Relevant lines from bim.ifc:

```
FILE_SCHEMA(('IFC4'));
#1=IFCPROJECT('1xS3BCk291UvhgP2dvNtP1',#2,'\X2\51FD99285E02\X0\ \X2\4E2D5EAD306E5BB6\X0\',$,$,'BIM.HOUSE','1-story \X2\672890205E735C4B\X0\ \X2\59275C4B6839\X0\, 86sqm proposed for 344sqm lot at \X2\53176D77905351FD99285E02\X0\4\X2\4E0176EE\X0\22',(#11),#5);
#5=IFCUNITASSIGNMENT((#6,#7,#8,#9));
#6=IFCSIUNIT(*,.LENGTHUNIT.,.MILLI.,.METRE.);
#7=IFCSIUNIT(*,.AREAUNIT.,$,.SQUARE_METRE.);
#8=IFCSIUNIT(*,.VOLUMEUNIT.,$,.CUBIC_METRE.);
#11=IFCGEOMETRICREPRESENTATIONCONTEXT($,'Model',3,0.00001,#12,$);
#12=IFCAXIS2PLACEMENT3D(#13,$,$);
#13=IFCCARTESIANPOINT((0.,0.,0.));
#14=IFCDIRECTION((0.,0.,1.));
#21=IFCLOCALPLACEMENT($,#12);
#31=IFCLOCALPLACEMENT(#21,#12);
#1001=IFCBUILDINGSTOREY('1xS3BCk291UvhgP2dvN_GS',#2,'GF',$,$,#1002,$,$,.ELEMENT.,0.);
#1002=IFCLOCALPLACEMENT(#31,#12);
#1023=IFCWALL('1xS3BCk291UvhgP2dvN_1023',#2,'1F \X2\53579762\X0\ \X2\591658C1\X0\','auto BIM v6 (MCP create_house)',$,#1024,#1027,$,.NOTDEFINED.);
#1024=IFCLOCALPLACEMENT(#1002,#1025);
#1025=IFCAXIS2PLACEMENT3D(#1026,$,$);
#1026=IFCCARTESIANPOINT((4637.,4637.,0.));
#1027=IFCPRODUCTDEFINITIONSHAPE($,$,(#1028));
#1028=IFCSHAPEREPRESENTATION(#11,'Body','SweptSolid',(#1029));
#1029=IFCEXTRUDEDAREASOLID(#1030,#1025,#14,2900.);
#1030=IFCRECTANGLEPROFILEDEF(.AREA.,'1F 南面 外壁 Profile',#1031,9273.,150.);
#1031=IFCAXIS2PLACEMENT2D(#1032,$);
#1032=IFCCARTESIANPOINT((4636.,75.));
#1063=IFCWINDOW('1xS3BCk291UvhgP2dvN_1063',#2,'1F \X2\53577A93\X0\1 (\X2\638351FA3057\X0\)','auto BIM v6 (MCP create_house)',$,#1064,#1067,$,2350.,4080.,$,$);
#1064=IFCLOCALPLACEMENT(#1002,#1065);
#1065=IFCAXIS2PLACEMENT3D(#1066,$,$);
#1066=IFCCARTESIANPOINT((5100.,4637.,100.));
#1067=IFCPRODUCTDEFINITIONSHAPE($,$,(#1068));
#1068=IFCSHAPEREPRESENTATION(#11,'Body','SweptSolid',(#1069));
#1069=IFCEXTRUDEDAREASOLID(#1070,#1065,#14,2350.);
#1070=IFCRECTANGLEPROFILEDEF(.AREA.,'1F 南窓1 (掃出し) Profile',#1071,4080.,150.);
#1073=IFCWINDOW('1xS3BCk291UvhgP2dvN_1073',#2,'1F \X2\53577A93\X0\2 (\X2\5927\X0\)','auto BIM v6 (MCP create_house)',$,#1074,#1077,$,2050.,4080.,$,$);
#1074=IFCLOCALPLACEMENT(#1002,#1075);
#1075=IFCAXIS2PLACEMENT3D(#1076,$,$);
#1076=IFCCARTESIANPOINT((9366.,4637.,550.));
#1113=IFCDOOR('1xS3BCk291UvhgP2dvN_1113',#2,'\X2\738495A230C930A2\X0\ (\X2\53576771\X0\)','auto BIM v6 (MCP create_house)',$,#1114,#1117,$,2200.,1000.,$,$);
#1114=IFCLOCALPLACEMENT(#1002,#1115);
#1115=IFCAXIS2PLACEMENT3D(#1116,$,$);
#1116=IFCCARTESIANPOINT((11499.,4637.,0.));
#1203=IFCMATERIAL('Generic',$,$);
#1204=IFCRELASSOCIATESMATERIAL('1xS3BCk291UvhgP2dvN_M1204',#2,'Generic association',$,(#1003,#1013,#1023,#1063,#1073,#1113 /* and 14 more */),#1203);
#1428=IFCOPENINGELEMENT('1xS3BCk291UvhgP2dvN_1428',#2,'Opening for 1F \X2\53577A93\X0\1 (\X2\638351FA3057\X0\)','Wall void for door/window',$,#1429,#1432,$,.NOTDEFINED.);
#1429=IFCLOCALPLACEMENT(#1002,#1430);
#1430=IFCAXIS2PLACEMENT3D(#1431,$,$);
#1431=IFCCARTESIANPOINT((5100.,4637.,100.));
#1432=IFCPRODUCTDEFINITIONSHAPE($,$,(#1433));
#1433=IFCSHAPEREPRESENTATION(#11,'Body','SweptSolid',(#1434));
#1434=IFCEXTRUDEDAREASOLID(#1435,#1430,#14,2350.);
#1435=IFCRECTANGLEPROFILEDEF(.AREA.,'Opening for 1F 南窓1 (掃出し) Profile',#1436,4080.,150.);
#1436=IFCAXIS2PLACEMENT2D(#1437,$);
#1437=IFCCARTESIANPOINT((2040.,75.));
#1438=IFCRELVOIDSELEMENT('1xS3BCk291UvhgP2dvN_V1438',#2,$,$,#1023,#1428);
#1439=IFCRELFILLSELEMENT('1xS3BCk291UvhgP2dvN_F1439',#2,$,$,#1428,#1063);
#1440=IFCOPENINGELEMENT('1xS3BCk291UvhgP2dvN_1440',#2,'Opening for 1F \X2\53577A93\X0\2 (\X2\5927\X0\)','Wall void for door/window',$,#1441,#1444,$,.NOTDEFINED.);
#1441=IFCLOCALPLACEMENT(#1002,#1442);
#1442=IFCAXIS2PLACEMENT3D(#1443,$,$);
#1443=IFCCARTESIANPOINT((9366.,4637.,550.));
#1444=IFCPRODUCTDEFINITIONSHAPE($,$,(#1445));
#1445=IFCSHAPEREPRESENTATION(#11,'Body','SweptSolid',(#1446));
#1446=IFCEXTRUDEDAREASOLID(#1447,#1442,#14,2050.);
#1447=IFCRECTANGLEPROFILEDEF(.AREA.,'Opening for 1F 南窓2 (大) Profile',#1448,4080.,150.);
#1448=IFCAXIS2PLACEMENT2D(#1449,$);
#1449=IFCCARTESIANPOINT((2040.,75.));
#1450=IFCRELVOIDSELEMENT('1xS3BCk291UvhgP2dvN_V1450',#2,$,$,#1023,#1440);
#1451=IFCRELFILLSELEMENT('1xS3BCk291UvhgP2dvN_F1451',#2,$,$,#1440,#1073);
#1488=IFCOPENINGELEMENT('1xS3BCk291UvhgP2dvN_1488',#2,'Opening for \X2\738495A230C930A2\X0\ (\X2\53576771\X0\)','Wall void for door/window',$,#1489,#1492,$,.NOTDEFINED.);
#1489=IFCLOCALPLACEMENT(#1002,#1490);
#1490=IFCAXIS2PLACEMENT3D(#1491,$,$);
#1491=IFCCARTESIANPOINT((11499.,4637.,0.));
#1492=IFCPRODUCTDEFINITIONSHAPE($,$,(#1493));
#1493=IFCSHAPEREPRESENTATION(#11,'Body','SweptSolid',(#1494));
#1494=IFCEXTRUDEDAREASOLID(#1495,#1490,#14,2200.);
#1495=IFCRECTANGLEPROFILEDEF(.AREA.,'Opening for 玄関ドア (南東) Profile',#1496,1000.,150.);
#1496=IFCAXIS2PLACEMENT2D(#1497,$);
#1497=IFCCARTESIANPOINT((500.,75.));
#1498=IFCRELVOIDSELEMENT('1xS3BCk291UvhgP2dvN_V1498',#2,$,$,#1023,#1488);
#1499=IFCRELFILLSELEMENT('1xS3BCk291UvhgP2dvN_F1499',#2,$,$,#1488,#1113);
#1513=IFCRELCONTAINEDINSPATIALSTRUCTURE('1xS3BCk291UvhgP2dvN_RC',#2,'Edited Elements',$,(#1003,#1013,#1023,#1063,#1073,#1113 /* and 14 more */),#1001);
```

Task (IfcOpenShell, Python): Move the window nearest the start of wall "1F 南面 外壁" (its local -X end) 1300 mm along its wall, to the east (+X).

```python
import ifcopenshell
import ifcopenshell.api.geometry
import ifcopenshell.util.placement
import ifcopenshell.util.unit

model = ifcopenshell.open("bim.ifc")
unit_scale = ifcopenshell.util.unit.calculate_unit_scale(model)

window = model.by_id(1063)
opening = window.FillsVoids[0].RelatingOpeningElement
wall = opening.VoidsElements[0].RelatingBuildingElement

wall_matrix = ifcopenshell.util.placement.get_local_placement(wall.ObjectPlacement)
shift = wall_matrix[:3, 0] * 1.3 / unit_scale
before = ifcopenshell.util.placement.get_local_placement(window.ObjectPlacement)[:3, 3].copy()

# The window is not placed relative to its opening, so move both.
for product in (opening, window):
    matrix = ifcopenshell.util.placement.get_local_placement(product.ObjectPlacement)
    matrix[:3, 3] += shift
    ifcopenshell.api.geometry.edit_object_placement(model, product=product, matrix=matrix, is_si=False)

after = ifcopenshell.util.placement.get_local_placement(window.ObjectPlacement)[:3, 3]
print("window moved by", (after - before).round(3) + 0.0)

model.write("bim-out.ifc")
```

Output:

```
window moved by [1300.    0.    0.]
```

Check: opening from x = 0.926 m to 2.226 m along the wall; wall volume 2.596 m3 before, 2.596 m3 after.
